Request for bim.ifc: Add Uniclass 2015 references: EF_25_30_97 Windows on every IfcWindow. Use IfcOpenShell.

First a look at what the model holds.

```python
import ifcopenshell

model = ifcopenshell.open("bim.ifc")
print(model.schema)
print("classifications:", [c.Name for c in model.by_type("IfcClassification")])
for ifc_class in ("IfcDoor", "IfcRoof", "IfcStair", "IfcWall", "IfcWindow"):
    print(ifc_class, len(model.by_type(ifc_class)))
```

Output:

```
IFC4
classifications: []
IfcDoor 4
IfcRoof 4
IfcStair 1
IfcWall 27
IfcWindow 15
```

```python
import ifcopenshell
import ifcopenshell.api.classification

model = ifcopenshell.open("bim.ifc")

system = ifcopenshell.api.classification.add_classification(model, classification="Uniclass 2015")

codes = {
    "IfcWindow": ("EF_25_30_97", "Windows"),
}
for ifc_class, (code, name) in codes.items():
    products = model.by_type(ifc_class)
    ifcopenshell.api.classification.add_reference(
        model, products=products, classification=system, identification=code, name=name
    )
    print(code, len(products))

model.write("bim-out.ifc")
```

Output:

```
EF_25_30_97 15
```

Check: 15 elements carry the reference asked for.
